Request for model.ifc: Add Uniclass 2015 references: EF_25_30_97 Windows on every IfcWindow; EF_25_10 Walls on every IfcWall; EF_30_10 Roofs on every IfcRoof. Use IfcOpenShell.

First a look at what the model holds.

```python
import ifcopenshell

model = ifcopenshell.open("model.ifc")
print(model.schema)
print("classifications:", [c.Name for c in model.by_type("IfcClassification")])
for ifc_class in ("IfcDoor", "IfcRoof", "IfcStair", "IfcWall", "IfcWindow"):
    print(ifc_class, len(model.by_type(ifc_class)))
```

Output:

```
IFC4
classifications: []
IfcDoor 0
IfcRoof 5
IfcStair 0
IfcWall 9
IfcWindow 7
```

```python
import ifcopenshell
import ifcopenshell.api.classification

model = ifcopenshell.open("model.ifc")

system = ifcopenshell.api.classification.add_classification(model, classification="Uniclass 2015")

codes = {
    "IfcWindow": ("EF_25_30_97", "Windows"),
    "IfcWall": ("EF_25_10", "Walls"),
    "IfcRoof": ("EF_30_10", "Roofs"),
}
for ifc_class, (code, name) in codes.items():
    products = model.by_type(ifc_class)
    ifcopenshell.api.classification.add_reference(
        model, products=products, classification=system, identification=code, name=name
    )
    print(code, len(products))

model.write("model_rev.ifc")
```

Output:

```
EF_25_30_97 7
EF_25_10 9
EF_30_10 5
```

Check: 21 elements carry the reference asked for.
